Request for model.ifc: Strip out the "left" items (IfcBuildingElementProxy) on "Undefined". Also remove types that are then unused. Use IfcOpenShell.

First a look at what the model holds.

```python
import ifcopenshell
import ifcopenshell.util.element

model = ifcopenshell.open("model.ifc")
print(model.schema)
storey = next(s for s in model.by_type("IfcBuildingStorey") if s.Name == "Undefined")
proxies = [e for e in ifcopenshell.util.element.get_decomposition(storey) if e.is_a("IfcBuildingElementProxy")]
seen = {}
for e in proxies:
    element_type = ifcopenshell.util.element.get_type(e)
    name = element_type.Name if element_type not in (None, e) else None
    seen[name] = seen.get(name, 0) + 1
for name, count in sorted(seen.items(), key=str):
    print(count, "x", name)
```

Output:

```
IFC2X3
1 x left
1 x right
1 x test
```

```python
import ifcopenshell
import ifcopenshell.api.root
import ifcopenshell.util.element

model = ifcopenshell.open("model.ifc")

storey = next(s for s in model.by_type("IfcBuildingStorey") if s.Name == "Undefined")
proxies = [e for e in ifcopenshell.util.element.get_decomposition(storey) if e.is_a("IfcBuildingElementProxy")]
targets = [e for e in proxies if (t := ifcopenshell.util.element.get_type(e)) not in (None, e) and t.Name == "left"]
types = {ifcopenshell.util.element.get_type(e) for e in targets} - {None, *targets}

for e in targets:
    ifcopenshell.api.root.remove_product(model, product=e)
print(len(targets), "removed")

unused = [t for t in types if not ifcopenshell.util.element.get_types(t)]
for t in unused:
    ifcopenshell.api.root.remove_product(model, product=t)
print(len(unused), "unused types removed")

model.write("model-out.ifc")
```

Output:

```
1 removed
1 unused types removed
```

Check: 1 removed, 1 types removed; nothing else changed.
